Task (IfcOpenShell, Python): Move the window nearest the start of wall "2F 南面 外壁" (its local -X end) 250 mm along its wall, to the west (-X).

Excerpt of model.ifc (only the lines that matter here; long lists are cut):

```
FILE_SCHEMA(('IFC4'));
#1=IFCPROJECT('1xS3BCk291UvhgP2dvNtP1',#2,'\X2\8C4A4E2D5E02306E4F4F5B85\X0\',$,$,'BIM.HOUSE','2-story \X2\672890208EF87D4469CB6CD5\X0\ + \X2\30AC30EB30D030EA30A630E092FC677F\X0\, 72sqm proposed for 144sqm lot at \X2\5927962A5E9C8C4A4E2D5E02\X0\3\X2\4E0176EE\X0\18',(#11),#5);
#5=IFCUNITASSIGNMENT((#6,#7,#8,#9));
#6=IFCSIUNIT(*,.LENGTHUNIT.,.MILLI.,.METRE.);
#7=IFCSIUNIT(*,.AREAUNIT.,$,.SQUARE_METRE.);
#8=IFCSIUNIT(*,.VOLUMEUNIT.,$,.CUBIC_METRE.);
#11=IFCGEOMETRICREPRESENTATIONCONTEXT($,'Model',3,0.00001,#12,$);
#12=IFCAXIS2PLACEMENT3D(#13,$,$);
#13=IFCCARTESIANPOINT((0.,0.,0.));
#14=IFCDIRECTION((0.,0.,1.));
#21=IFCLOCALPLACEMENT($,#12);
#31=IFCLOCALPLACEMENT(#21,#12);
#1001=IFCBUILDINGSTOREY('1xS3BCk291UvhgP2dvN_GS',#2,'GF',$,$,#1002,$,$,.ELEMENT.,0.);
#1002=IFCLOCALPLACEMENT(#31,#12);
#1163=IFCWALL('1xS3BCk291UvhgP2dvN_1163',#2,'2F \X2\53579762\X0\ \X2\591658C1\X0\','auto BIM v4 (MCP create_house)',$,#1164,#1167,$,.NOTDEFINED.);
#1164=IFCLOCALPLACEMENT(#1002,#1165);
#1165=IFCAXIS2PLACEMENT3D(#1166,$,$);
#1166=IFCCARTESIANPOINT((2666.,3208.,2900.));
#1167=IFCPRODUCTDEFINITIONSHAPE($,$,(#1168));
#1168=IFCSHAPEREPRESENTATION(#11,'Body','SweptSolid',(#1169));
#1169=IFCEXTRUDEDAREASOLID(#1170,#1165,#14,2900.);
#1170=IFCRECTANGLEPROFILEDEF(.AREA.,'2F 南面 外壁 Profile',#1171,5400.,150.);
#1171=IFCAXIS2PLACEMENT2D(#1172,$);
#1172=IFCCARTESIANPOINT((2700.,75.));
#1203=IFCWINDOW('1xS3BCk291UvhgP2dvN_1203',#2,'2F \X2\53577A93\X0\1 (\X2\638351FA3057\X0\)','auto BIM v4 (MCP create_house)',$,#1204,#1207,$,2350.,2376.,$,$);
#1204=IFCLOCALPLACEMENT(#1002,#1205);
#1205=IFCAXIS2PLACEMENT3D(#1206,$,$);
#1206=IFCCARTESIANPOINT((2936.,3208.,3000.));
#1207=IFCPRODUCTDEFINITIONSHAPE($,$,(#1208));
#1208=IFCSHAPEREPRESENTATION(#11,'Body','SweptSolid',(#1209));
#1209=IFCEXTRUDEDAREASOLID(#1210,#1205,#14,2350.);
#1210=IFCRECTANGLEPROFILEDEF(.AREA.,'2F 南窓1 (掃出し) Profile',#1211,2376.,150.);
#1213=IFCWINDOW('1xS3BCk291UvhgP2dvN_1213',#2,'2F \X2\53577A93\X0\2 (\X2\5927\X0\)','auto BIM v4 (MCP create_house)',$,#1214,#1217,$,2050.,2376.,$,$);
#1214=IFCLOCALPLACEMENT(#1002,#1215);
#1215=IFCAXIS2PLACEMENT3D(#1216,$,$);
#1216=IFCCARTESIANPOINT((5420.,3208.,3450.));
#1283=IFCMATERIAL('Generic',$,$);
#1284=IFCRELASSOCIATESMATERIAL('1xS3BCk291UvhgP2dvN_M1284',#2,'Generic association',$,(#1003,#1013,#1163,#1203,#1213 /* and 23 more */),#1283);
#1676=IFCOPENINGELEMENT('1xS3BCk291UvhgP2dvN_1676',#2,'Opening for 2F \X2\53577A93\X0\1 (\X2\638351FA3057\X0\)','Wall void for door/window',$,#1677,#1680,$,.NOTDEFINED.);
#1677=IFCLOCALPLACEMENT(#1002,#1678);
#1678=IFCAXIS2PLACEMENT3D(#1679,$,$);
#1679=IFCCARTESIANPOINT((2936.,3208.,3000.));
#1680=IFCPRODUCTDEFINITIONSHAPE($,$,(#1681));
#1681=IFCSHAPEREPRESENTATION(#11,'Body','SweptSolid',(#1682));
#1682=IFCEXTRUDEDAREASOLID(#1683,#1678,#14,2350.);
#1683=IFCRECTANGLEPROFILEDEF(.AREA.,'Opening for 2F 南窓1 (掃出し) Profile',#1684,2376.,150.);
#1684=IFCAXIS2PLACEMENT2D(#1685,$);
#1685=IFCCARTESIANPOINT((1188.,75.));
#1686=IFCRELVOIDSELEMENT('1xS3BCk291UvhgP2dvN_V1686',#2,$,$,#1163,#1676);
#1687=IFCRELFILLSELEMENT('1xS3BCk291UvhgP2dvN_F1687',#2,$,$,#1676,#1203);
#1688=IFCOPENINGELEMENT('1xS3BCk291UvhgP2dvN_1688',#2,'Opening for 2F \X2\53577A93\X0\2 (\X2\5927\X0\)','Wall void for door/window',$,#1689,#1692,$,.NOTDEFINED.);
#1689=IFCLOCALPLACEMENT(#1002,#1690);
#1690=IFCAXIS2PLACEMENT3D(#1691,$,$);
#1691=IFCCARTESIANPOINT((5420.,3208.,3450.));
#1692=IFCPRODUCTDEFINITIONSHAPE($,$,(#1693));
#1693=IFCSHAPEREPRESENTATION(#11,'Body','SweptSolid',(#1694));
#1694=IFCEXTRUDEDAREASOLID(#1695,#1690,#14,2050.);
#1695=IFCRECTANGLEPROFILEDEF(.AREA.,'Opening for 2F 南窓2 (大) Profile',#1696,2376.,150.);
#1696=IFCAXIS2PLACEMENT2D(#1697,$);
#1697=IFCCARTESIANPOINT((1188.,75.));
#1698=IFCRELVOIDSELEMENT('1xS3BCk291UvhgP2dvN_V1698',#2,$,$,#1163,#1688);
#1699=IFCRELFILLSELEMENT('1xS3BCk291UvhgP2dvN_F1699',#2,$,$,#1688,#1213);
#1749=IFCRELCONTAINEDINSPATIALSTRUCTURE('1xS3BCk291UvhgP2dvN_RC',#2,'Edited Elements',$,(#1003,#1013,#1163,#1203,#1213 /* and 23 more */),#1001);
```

```python
import ifcopenshell
import ifcopenshell.api.geometry
import ifcopenshell.util.placement
import ifcopenshell.util.unit

model = ifcopenshell.open("model.ifc")
unit_scale = ifcopenshell.util.unit.calculate_unit_scale(model)

window = model.by_id(1203)
opening = window.FillsVoids[0].RelatingOpeningElement
wall = opening.VoidsElements[0].RelatingBuildingElement

wall_matrix = ifcopenshell.util.placement.get_local_placement(wall.ObjectPlacement)
shift = wall_matrix[:3, 0] * -0.25 / unit_scale
before = ifcopenshell.util.placement.get_local_placement(window.ObjectPlacement)[:3, 3].copy()

# The window is not placed relative to its opening, so move both.
for product in (opening, window):
    matrix = ifcopenshell.util.placement.get_local_placement(product.ObjectPlacement)
    matrix[:3, 3] += shift
    ifcopenshell.api.geometry.edit_object_placement(model, product=product, matrix=matrix, is_si=False)

after = ifcopenshell.util.placement.get_local_placement(window.ObjectPlacement)[:3, 3]
print("window moved by", (after - before).round(3) + 0.0)

model.write("model-out.ifc")
```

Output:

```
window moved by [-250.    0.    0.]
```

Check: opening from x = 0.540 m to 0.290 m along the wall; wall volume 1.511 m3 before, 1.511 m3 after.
